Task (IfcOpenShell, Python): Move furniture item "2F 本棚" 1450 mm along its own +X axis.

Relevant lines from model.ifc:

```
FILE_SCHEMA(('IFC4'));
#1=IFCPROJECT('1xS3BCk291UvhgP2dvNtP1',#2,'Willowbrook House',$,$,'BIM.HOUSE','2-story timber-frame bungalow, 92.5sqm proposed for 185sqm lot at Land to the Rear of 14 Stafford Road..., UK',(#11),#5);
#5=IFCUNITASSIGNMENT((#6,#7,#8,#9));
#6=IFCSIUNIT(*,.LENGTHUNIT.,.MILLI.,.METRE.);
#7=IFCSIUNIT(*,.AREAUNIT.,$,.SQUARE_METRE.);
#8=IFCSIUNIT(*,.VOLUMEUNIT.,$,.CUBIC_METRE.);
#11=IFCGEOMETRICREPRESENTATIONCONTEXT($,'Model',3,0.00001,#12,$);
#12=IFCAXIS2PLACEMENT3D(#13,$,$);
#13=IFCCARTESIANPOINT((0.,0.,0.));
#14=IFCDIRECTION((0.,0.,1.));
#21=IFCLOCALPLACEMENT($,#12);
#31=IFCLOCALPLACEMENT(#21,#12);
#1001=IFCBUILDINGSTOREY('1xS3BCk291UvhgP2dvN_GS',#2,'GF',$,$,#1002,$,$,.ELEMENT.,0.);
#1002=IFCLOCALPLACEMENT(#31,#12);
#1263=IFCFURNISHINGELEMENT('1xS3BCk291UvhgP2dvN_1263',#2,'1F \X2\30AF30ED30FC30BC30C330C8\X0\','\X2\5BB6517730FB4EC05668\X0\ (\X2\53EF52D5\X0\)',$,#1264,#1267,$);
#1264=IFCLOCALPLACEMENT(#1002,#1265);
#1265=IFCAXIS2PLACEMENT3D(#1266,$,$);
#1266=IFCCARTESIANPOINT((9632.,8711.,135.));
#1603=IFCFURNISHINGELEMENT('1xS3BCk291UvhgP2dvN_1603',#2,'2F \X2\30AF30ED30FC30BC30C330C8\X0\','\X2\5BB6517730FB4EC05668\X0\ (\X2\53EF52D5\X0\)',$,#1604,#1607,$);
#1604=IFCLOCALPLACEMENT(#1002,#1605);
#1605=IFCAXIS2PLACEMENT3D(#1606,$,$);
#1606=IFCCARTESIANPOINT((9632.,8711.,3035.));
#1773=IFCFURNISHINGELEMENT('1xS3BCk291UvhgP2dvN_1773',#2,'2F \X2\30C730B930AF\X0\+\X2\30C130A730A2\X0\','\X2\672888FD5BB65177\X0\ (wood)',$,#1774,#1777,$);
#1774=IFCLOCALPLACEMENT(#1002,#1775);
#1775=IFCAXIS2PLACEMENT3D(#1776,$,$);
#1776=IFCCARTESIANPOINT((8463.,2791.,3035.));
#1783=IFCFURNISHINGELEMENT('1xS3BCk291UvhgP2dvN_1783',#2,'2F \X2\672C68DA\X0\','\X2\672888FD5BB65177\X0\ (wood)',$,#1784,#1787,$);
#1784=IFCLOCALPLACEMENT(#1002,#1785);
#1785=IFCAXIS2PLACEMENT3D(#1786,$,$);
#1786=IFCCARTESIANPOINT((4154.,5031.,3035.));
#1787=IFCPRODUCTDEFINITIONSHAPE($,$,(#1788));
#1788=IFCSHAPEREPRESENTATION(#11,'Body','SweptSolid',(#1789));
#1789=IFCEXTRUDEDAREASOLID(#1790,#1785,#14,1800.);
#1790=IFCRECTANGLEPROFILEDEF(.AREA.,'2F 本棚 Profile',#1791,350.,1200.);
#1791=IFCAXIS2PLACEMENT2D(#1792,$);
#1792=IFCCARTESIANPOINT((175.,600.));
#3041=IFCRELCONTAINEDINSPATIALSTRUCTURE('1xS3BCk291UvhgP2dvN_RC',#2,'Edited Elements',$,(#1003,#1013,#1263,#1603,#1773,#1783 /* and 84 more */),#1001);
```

```python
import ifcopenshell
import ifcopenshell.api.geometry
import ifcopenshell.util.placement

model = ifcopenshell.open("model.ifc")

item = model.by_guid("1xS3BCk291UvhgP2dvN_1783")
matrix = ifcopenshell.util.placement.get_local_placement(item.ObjectPlacement)
matrix[:3, 3] += matrix[:3, 0] * 1450.0
ifcopenshell.api.geometry.edit_object_placement(model, product=item, matrix=matrix, is_si=False)

print(ifcopenshell.util.placement.get_local_placement(item.ObjectPlacement).round(3) + 0.0)

model.write("model_rev.ifc")
```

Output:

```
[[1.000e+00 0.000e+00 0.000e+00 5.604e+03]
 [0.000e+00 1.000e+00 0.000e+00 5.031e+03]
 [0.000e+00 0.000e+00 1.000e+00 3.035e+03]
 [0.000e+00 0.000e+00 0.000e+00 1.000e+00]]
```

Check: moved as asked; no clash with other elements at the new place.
